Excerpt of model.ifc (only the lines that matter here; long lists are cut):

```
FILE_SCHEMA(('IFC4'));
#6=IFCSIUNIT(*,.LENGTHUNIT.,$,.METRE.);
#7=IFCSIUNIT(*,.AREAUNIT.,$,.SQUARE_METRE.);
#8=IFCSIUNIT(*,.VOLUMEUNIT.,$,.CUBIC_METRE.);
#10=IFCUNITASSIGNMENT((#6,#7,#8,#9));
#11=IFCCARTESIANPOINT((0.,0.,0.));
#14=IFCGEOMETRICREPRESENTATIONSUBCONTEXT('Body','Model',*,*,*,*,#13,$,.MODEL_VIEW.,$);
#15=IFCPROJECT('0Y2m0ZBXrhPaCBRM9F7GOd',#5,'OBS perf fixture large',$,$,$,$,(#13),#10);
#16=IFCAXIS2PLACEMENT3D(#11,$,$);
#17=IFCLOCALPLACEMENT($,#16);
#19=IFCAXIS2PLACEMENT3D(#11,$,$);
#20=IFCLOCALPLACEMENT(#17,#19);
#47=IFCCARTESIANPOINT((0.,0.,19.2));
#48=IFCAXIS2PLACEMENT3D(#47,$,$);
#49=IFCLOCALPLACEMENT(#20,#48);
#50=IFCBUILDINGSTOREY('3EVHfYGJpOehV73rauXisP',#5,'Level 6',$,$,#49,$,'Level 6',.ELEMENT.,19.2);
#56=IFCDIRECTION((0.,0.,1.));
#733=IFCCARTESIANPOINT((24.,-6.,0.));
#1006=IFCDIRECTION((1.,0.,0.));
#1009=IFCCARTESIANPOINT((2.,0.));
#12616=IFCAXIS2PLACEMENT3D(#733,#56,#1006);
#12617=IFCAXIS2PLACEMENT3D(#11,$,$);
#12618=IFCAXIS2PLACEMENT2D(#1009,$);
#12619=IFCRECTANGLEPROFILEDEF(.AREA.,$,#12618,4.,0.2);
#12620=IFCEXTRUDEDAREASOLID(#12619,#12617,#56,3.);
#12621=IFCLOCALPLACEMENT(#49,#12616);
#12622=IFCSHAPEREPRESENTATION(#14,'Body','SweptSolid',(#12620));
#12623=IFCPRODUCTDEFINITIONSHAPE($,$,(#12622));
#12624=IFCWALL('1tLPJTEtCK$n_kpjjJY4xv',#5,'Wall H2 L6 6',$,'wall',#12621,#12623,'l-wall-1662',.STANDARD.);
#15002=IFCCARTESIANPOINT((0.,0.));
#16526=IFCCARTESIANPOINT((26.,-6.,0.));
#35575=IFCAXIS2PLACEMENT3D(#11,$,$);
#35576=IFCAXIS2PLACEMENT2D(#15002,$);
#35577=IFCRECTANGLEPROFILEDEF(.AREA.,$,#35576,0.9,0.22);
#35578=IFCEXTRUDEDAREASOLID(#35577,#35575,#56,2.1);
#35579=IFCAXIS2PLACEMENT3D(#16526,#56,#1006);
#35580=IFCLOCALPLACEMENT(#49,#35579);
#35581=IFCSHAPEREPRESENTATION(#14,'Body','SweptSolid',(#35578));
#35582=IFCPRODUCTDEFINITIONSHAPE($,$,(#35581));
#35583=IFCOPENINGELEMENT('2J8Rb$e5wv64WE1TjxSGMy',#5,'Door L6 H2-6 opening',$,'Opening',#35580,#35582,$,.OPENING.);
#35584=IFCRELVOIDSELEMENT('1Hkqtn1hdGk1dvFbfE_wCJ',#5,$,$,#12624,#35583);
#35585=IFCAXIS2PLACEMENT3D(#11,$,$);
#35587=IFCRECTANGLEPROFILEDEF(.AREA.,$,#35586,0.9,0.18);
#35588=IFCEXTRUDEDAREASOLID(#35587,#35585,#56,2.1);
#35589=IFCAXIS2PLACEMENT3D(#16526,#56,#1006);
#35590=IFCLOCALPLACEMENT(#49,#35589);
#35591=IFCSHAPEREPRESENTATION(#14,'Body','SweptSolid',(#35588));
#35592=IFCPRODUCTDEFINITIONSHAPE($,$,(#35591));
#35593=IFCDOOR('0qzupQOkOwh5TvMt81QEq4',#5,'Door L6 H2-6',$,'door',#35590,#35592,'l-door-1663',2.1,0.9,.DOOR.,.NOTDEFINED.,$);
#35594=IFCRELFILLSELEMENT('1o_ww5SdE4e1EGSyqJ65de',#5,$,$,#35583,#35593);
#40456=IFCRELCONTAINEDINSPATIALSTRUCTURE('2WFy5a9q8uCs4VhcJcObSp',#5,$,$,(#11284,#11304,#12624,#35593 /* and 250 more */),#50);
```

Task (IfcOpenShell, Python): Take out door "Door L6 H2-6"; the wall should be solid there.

```python
import ifcopenshell
import ifcopenshell.api.feature
import ifcopenshell.api.root
import ifcopenshell.geom
import ifcopenshell.util.shape

model = ifcopenshell.open("model.ifc")
settings = ifcopenshell.geom.settings()


def volume(element):
    """Net volume in cubic metres, openings subtracted."""
    shape = ifcopenshell.geom.create_shape(settings, element)
    return ifcopenshell.util.shape.get_volume(shape.geometry)


door = model.by_guid("0qzupQOkOwh5TvMt81QEq4")
opening = door.FillsVoids[0].RelatingOpeningElement
wall = opening.VoidsElements[0].RelatingBuildingElement
before = volume(wall)

ifcopenshell.api.root.remove_product(model, product=door)
ifcopenshell.api.feature.remove_feature(model, feature=opening)

after = volume(wall)

print(f"wall volume {before:.3f} -> {after:.3f} m3")

model.write("model-out.ifc")
```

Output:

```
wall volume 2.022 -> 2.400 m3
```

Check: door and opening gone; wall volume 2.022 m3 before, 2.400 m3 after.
